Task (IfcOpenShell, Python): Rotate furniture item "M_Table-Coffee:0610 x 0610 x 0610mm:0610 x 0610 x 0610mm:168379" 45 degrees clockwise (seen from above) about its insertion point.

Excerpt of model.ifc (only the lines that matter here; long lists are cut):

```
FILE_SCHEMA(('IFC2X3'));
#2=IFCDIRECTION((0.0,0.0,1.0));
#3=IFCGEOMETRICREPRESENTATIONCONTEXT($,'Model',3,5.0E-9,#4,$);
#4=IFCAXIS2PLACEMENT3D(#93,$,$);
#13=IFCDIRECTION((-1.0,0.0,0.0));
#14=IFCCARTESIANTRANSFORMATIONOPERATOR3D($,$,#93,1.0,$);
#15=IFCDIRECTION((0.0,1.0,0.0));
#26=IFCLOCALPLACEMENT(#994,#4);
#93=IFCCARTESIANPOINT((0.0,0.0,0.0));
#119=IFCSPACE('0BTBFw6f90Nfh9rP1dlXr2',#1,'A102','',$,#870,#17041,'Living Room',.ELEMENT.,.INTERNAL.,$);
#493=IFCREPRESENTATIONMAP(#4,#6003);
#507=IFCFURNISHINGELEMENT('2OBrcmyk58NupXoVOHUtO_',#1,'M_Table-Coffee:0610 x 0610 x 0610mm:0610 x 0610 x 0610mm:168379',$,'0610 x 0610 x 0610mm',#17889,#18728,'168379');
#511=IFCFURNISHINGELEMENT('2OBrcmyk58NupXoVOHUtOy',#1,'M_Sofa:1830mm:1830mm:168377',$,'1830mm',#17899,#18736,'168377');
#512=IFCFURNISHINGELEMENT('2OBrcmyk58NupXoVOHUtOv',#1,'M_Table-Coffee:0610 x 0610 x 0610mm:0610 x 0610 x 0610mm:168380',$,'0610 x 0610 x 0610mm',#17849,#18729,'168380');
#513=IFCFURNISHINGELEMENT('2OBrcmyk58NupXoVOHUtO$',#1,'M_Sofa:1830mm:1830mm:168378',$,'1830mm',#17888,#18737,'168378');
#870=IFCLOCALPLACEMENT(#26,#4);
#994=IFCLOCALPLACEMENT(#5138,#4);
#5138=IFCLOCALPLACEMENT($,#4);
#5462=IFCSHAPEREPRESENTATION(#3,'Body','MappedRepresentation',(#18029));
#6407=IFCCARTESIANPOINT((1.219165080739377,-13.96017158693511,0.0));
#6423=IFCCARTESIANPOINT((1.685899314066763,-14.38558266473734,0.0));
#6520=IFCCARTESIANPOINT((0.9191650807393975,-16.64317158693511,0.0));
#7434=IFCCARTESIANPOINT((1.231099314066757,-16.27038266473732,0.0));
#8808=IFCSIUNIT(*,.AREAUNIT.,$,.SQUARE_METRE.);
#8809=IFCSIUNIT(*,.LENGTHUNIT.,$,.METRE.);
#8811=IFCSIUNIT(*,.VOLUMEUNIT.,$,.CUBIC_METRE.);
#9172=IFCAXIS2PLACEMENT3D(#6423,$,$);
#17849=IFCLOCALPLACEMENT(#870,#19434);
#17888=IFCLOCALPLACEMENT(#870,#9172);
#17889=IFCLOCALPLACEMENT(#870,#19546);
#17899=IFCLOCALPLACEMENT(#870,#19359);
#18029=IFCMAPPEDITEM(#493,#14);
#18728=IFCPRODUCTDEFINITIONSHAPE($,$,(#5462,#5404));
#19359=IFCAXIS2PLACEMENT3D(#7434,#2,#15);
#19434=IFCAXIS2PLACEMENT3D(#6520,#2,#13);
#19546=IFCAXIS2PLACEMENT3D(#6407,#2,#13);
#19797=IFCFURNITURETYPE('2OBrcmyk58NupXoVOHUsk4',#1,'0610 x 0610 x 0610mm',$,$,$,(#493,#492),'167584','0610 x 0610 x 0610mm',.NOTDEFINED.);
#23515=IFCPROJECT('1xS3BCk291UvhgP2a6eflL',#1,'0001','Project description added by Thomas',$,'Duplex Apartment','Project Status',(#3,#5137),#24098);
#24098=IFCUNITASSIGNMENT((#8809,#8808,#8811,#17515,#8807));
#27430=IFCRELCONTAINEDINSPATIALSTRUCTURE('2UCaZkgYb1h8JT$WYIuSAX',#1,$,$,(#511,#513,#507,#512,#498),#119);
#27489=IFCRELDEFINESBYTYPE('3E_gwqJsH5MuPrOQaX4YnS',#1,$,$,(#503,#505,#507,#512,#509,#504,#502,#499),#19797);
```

```python
import ifcopenshell
import ifcopenshell.api.geometry
import ifcopenshell.util.placement

model = ifcopenshell.open("model.ifc")

item = model.by_guid("2OBrcmyk58NupXoVOHUtO_")
matrix = ifcopenshell.util.placement.get_local_placement(item.ObjectPlacement)
matrix = matrix @ ifcopenshell.util.placement.rotation(-45, "Z")
ifcopenshell.api.geometry.edit_object_placement(model, product=item, matrix=matrix, is_si=False)

print(ifcopenshell.util.placement.get_local_placement(item.ObjectPlacement).round(3) + 0.0)

model.write("model_rev.ifc")
```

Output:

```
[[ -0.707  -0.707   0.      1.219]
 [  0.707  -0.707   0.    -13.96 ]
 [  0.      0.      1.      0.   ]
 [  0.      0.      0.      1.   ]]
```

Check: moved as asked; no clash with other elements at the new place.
